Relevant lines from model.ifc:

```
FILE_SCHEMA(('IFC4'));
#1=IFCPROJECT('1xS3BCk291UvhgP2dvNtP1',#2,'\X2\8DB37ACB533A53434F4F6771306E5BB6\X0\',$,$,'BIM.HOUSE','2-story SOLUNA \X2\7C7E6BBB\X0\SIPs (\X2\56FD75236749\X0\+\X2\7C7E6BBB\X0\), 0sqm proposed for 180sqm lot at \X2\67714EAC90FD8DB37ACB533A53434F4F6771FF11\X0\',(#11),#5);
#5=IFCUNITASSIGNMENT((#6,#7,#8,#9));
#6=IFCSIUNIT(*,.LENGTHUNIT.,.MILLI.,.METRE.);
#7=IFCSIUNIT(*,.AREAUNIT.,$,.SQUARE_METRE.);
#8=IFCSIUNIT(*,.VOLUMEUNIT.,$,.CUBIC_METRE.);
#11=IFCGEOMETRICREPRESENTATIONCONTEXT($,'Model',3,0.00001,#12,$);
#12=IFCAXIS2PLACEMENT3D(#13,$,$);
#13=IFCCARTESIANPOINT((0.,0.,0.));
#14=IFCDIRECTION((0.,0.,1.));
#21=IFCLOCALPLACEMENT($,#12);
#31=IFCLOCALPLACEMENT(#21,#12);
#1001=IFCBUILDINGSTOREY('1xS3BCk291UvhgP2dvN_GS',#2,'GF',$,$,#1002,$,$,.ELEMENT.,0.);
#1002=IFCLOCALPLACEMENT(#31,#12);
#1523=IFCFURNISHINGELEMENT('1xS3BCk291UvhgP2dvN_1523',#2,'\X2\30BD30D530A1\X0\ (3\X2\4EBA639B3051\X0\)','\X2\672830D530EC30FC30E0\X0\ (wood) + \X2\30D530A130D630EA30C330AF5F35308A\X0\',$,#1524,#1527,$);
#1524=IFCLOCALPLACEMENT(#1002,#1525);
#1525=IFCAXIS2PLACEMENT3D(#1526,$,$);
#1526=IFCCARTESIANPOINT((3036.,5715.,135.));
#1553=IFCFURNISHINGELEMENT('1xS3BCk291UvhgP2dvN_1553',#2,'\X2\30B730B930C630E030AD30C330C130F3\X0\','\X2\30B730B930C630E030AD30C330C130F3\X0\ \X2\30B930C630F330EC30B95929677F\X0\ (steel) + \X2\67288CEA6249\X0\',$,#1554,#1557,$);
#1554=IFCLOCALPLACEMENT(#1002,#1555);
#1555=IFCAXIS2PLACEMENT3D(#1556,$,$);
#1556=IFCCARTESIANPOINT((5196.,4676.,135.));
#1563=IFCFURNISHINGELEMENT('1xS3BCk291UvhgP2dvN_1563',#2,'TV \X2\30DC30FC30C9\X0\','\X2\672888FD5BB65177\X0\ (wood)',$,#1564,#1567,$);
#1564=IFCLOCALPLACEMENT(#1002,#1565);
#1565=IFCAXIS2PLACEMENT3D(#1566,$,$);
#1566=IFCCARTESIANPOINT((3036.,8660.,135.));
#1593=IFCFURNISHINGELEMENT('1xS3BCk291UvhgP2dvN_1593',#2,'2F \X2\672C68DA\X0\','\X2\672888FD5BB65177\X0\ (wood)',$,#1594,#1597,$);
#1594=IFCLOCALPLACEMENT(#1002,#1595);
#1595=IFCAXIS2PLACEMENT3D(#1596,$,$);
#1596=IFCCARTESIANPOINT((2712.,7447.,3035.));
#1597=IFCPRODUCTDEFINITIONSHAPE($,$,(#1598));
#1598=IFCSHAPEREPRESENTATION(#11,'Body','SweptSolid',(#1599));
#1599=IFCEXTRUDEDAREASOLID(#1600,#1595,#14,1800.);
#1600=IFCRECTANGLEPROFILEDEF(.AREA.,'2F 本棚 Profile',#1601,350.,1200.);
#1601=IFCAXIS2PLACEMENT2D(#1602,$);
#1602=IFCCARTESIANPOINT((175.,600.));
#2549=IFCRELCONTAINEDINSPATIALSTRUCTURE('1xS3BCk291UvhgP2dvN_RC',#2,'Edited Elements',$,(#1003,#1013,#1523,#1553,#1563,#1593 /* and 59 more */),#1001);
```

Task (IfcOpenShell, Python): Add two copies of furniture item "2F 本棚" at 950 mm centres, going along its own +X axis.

```python
import ifcopenshell
import ifcopenshell.api.geometry
import ifcopenshell.api.root
import ifcopenshell.util.element
import ifcopenshell.util.placement
import ifcopenshell.util.unit

model = ifcopenshell.open("model.ifc")
unit_scale = ifcopenshell.util.unit.calculate_unit_scale(model)


def reuse_history(source, copy):
    """copy_class also copies each property set's owner history, people and application; keep the originals."""
    for rel in copy.IsDefinedBy:
        if rel.is_a("IfcRelDefinesByProperties") and (history := rel.RelatingPropertyDefinition.OwnerHistory):
            rel.RelatingPropertyDefinition.OwnerHistory = source.OwnerHistory
            ifcopenshell.util.element.remove_deep2(model, history)


source = model.by_id(1593)
base = ifcopenshell.util.placement.get_local_placement(source.ObjectPlacement)
step = base[:3, 0] * 0.95 / unit_scale

for i in range(1, 3):
    copy = ifcopenshell.api.root.copy_class(model, product=source)
    copy.Representation = ifcopenshell.util.element.copy_deep(
        model, source.Representation, exclude=["IfcGeometricRepresentationContext", "IfcRepresentationMap"]
    )
    reuse_history(source, copy)
    matrix = base.copy()
    matrix[:3, 3] += i * step
    print("added at", matrix[:3, 3].round(3) + 0.0)
    ifcopenshell.api.geometry.edit_object_placement(model, product=copy, matrix=matrix, is_si=False)

model.write("model-out.ifc")
```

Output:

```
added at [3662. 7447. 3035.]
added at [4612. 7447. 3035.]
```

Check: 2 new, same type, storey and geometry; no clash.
